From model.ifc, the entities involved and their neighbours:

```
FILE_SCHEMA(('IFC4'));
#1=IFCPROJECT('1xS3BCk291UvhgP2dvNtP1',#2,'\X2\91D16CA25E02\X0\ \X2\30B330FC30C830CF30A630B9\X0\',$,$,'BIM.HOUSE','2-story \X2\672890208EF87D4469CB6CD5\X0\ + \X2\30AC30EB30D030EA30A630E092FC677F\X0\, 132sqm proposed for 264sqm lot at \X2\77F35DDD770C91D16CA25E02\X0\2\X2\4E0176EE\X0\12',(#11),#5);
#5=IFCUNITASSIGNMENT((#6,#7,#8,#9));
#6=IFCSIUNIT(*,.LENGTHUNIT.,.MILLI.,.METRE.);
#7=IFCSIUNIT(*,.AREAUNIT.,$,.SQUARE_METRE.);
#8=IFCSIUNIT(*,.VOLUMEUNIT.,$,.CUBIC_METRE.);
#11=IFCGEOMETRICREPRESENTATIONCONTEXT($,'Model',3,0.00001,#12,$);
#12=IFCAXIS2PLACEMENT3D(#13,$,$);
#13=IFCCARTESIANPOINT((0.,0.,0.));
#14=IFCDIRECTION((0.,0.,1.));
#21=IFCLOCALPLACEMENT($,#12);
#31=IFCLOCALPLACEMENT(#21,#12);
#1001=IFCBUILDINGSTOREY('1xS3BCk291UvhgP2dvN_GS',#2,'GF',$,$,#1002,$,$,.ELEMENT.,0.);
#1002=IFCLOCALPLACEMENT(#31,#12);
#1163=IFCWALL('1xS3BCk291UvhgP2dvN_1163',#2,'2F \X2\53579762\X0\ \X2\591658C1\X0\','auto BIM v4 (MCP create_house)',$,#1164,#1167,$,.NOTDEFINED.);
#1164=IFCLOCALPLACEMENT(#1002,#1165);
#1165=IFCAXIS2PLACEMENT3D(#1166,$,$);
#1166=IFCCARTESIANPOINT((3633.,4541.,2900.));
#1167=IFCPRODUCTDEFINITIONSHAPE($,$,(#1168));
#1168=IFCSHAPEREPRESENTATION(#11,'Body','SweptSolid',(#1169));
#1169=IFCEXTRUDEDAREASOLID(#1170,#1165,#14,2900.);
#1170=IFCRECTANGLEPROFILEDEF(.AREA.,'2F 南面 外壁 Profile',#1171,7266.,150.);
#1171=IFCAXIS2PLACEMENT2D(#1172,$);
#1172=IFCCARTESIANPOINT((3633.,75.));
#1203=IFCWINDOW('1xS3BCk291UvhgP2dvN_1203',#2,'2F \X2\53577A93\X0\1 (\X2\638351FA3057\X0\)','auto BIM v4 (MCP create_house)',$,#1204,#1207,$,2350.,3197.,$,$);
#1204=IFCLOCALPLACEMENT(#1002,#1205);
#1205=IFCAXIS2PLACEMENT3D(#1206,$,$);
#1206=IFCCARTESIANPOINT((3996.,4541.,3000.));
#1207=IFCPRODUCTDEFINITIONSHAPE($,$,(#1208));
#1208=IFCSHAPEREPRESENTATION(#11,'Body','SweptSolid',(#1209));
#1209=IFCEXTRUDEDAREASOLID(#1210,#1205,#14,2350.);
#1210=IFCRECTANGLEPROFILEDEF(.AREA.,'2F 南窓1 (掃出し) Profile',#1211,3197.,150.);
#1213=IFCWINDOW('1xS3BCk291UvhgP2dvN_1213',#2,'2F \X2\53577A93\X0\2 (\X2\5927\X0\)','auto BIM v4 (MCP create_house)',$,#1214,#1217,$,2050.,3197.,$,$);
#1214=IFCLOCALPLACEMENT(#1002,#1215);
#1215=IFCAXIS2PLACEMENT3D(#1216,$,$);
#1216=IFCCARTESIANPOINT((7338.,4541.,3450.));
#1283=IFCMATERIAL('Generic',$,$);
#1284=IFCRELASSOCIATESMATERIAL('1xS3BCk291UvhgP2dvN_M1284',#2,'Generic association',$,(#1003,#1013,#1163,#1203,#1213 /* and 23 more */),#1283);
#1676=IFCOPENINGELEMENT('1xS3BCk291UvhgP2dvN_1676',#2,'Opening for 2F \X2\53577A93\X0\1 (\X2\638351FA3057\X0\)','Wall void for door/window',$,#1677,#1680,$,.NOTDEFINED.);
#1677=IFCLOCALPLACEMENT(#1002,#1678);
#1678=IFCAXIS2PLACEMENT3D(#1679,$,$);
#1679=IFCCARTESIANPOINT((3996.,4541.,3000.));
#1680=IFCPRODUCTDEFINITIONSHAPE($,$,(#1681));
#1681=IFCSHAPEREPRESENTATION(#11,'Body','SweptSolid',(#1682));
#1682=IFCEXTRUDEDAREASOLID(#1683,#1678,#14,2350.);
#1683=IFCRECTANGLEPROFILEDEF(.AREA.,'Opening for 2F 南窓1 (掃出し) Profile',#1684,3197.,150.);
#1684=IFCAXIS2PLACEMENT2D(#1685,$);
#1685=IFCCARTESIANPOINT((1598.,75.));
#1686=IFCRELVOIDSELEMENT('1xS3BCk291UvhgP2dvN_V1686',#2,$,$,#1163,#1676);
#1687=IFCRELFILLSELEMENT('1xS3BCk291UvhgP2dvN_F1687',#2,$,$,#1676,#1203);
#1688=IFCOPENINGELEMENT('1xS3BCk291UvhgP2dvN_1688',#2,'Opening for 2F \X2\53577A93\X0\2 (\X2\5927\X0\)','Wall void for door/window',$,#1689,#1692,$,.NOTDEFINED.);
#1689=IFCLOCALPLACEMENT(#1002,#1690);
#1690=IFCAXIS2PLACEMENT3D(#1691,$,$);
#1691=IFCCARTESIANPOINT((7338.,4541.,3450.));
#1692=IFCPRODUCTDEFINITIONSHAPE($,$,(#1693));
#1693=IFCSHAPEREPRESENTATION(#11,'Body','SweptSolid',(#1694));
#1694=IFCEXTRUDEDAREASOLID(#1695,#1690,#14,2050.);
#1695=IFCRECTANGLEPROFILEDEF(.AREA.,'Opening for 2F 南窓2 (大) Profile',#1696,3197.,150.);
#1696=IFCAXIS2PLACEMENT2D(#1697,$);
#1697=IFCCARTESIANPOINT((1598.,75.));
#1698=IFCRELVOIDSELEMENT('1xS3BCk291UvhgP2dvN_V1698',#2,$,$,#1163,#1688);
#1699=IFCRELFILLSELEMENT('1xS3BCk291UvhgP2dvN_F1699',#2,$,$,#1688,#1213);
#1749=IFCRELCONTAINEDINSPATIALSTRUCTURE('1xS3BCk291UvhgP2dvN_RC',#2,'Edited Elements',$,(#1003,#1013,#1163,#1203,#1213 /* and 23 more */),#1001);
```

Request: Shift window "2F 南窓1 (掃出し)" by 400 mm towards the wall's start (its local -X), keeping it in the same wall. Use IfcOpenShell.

```python
import ifcopenshell
import ifcopenshell.api.geometry
import ifcopenshell.util.placement
import ifcopenshell.util.unit

model = ifcopenshell.open("model.ifc")
unit_scale = ifcopenshell.util.unit.calculate_unit_scale(model)

window = model.by_id(1203)
opening = window.FillsVoids[0].RelatingOpeningElement
wall = opening.VoidsElements[0].RelatingBuildingElement

wall_matrix = ifcopenshell.util.placement.get_local_placement(wall.ObjectPlacement)
shift = wall_matrix[:3, 0] * -0.4 / unit_scale
before = ifcopenshell.util.placement.get_local_placement(window.ObjectPlacement)[:3, 3].copy()

# The window is not placed relative to its opening, so move both.
for product in (opening, window):
    matrix = ifcopenshell.util.placement.get_local_placement(product.ObjectPlacement)
    matrix[:3, 3] += shift
    ifcopenshell.api.geometry.edit_object_placement(model, product=product, matrix=matrix, is_si=False)

after = ifcopenshell.util.placement.get_local_placement(window.ObjectPlacement)[:3, 3]
print("window moved by", (after - before).round(3) + 0.0)

model.write("model_v2.ifc")
```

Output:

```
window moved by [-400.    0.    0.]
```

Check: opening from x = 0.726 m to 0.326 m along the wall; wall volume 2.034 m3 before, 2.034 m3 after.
